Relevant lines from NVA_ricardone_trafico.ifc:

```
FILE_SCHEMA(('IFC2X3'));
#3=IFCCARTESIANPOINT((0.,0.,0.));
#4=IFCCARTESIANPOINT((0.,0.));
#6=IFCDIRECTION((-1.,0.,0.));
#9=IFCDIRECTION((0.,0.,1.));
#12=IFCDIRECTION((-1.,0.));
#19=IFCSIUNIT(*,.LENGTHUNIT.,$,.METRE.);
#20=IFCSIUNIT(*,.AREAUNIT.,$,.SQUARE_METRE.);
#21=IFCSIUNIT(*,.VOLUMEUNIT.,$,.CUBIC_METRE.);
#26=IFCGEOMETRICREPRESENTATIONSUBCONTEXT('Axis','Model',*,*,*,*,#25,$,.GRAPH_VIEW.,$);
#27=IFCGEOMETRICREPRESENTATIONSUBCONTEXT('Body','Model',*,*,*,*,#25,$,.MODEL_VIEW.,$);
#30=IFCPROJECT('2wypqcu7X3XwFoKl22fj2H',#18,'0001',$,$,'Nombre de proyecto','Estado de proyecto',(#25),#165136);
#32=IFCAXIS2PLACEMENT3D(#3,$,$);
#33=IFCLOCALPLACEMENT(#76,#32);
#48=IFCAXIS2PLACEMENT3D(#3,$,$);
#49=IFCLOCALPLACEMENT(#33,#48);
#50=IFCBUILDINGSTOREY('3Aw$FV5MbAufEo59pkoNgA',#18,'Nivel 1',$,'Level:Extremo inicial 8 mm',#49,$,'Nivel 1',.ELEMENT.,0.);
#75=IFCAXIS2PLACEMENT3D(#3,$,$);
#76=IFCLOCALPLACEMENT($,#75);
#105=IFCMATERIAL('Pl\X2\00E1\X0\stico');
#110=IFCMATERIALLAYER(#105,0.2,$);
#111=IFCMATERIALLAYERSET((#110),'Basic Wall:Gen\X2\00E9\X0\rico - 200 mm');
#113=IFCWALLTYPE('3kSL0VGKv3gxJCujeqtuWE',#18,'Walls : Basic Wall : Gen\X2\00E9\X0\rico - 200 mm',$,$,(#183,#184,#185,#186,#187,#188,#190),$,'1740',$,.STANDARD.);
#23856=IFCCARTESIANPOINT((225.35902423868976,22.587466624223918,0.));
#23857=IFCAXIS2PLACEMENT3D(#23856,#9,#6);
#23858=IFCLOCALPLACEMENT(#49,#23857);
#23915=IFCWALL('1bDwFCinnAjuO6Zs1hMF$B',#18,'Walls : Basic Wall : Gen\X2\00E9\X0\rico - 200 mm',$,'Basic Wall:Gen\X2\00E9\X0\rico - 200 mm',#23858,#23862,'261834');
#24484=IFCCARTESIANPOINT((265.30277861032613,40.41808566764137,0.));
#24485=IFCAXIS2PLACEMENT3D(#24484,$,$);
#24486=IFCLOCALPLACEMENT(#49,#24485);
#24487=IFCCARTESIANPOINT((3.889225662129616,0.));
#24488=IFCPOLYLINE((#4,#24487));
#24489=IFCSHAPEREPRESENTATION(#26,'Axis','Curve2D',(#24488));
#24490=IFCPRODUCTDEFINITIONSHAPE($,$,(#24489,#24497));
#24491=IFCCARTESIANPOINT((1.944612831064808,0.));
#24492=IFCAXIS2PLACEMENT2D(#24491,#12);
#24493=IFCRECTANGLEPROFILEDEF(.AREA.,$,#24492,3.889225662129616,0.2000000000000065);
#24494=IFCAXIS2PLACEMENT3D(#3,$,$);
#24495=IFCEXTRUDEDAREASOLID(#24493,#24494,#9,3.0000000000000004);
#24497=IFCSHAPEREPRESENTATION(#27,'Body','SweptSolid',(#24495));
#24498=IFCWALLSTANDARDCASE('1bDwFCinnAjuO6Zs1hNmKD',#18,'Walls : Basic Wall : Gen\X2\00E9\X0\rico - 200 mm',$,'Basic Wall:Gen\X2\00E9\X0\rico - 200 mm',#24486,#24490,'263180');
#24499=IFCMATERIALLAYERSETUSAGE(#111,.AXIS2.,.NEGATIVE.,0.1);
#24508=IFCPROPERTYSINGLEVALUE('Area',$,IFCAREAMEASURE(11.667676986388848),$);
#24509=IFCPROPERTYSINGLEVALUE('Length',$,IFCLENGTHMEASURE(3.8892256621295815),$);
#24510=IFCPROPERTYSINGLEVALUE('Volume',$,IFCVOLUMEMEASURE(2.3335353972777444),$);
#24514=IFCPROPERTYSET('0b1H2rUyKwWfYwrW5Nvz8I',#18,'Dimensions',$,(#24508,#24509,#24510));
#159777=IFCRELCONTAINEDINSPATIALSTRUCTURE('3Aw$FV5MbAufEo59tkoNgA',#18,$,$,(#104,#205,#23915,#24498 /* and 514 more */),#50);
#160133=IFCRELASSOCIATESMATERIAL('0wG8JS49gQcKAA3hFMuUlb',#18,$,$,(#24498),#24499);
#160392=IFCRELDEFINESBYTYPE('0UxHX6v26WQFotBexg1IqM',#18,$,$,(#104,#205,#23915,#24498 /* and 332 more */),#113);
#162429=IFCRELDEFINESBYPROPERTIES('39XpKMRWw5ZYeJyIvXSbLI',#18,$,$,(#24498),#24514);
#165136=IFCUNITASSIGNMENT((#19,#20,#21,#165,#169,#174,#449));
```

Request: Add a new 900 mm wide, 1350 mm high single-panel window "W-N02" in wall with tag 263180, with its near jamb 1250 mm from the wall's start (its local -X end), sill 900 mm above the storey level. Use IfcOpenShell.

```python
import numpy as np
import ifcopenshell
import ifcopenshell.api.feature
import ifcopenshell.api.geometry
import ifcopenshell.api.pset
import ifcopenshell.api.root
import ifcopenshell.api.spatial
import ifcopenshell.api.type
import ifcopenshell.geom
import ifcopenshell.util.element
import ifcopenshell.util.placement
import ifcopenshell.util.representation
import ifcopenshell.util.shape
import ifcopenshell.util.unit

model = ifcopenshell.open("NVA_ricardone_trafico.ifc")
unit_scale = ifcopenshell.util.unit.calculate_unit_scale(model)
area_scale = ifcopenshell.util.unit.calculate_unit_scale(model, "AREAUNIT")
volume_scale = ifcopenshell.util.unit.calculate_unit_scale(model, "VOLUMEUNIT")
settings = ifcopenshell.geom.settings()


def volume(element):
    """Net volume in cubic metres, openings subtracted."""
    shape = ifcopenshell.geom.create_shape(settings, element)
    return ifcopenshell.util.shape.get_volume(shape.geometry)


wall = model.by_guid("1bDwFCinnAjuO6Zs1hNmKD")
storey = ifcopenshell.util.element.get_container(wall, ifc_class="IfcBuildingStorey")
context = ifcopenshell.util.representation.get_context(model, "Model", "Body", "MODEL_VIEW")
before = volume(wall)

width, height, from_end, sill = 0.9, 1.35, 1.25, 0.9  # metres

# The wall runs along its own X axis, and the end named is its -X end.
wall_shape = ifcopenshell.geom.create_shape(settings, wall)
x, y, z = ifcopenshell.util.shape.get_vertices(wall_shape.geometry).T
start = x.min() + from_end
face, thickness = float(y.min()), float(y.max() - y.min())
wall_matrix = ifcopenshell.util.placement.get_local_placement(wall.ObjectPlacement)
level = ifcopenshell.util.placement.get_local_placement(storey.ObjectPlacement)[2, 3]


def in_wall(x, y):
    """Placement at x, y metres in the wall's axes, at sill height."""
    matrix = wall_matrix.copy()
    matrix[:, 3] = wall_matrix @ np.array([x / unit_scale, y / unit_scale, 0.0, 1.0])
    matrix[2, 3] = level + sill / unit_scale
    return matrix


# Opening: a box that overshoots both wall faces by 50 mm.
opening = ifcopenshell.api.root.create_entity(model, ifc_class="IfcOpeningElement")
box = ifcopenshell.api.geometry.add_wall_representation(
    model, context=context, length=width, height=height, thickness=thickness + 0.1
)
ifcopenshell.api.geometry.assign_representation(model, product=opening, representation=box)
ifcopenshell.api.geometry.edit_object_placement(model, product=opening, matrix=in_wall(start, face - 0.05), is_si=False)
ifcopenshell.api.feature.add_feature(model, feature=opening, element=wall)

window = ifcopenshell.api.root.create_entity(model, ifc_class="IfcWindow", name="W-N02")
window.OverallWidth, window.OverallHeight = width / unit_scale, height / unit_scale
body = ifcopenshell.api.geometry.add_window_representation(
    model,
    context=context,
    overall_width=window.OverallWidth,
    overall_height=window.OverallHeight,
    partition_type="SINGLE_PANEL",
)
ifcopenshell.api.geometry.assign_representation(model, product=window, representation=body)
ifcopenshell.api.spatial.assign_container(model, products=[window], relating_structure=storey)
fills = ifcopenshell.api.feature.add_filling(model, opening=opening, element=window)
fills.OwnerHistory = window.OwnerHistory  # required in IFC2X3

# IFC2X3 keeps the operation on the window style.
style = ifcopenshell.api.root.create_entity(model, ifc_class="IfcWindowStyle", name="W-N02")
style.OperationType, style.ConstructionType = "SINGLE_PANEL", "NOTDEFINED"
style.ParameterTakesPrecedence = style.Sizeable = False
ifcopenshell.api.type.assign_type(model, related_objects=[window], relating_type=style)

# Centre the window in the wall's thickness.
ifcopenshell.api.geometry.edit_object_placement(model, product=window, matrix=in_wall(start, face), is_si=False)
window_shape = ifcopenshell.geom.create_shape(settings, window)
depth = ifcopenshell.util.shape.get_vertices(window_shape.geometry)[:, 1]
offset = face + thickness / 2 - (depth.min() + depth.max()) / 2
ifcopenshell.api.geometry.edit_object_placement(model, product=window, matrix=in_wall(start, offset), is_si=False)

after = volume(wall)

# Update the wall's stored quantities.
pset = model.by_id(ifcopenshell.util.element.get_pset(wall, "Dimensions", should_inherit=False)["id"])
ifcopenshell.api.pset.edit_pset(model, pset=pset, properties={
    "Area": model.create_entity("IfcAreaMeasure", after / thickness / area_scale),
    "Volume": model.create_entity("IfcVolumeMeasure", after / volume_scale),
})

print(f"wall volume {before:.3f} -> {after:.3f} m3")

model.write("NVA_ricardone_trafico_v2.ifc")
```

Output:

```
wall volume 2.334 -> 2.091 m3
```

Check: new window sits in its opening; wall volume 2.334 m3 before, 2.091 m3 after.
